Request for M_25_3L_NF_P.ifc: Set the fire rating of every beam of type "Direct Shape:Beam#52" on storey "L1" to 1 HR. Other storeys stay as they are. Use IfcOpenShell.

First a look at what the model holds.

```python
import ifcopenshell
import ifcopenshell.util.element

model = ifcopenshell.open("M_25_3L_NF_P.ifc")
print(model.schema)
storey = next(s for s in model.by_type("IfcBuildingStorey") if s.Name == "L1")
beams = [e for e in ifcopenshell.util.element.get_decomposition(storey) if e.is_a("IfcBeam")]
seen = {}
for e in beams:
    element_type = ifcopenshell.util.element.get_type(e)
    key = (element_type.Name if element_type != e and element_type else None, ifcopenshell.util.element.get_pset(e, "Pset_BeamCommon", "FireRating"))
    seen[key] = seen.get(key, 0) + 1
for (name, value), count in sorted(seen.items(), key=str):
    print(count, "x", name, "|", value)
```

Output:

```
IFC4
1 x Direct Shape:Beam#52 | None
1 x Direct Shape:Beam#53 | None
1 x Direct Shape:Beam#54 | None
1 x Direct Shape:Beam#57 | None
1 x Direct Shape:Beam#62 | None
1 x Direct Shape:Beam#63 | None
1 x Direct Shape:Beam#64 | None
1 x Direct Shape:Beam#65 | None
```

```python
import ifcopenshell
import ifcopenshell.api.pset
import ifcopenshell.util.element

model = ifcopenshell.open("M_25_3L_NF_P.ifc")

storey = next(s for s in model.by_type("IfcBuildingStorey") if s.Name == "L1")
beams = [e for e in ifcopenshell.util.element.get_decomposition(storey) if e.is_a("IfcBeam")]

count = 0
for e in beams:
    element_type = ifcopenshell.util.element.get_type(e)
    if element_type in (None, e) or element_type.Name != "Direct Shape:Beam#52":
        continue
    # add_pset returns the element's existing set when there is one.
    pset = ifcopenshell.api.pset.add_pset(model, product=e, name="Pset_BeamCommon")
    ifcopenshell.api.pset.edit_pset(model, pset=pset, properties={"FireRating": "1 HR"})
    count += 1

print(count, "beams updated")

model.write("M_25_3L_NF_P-out.ifc")
```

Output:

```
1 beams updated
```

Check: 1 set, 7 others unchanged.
